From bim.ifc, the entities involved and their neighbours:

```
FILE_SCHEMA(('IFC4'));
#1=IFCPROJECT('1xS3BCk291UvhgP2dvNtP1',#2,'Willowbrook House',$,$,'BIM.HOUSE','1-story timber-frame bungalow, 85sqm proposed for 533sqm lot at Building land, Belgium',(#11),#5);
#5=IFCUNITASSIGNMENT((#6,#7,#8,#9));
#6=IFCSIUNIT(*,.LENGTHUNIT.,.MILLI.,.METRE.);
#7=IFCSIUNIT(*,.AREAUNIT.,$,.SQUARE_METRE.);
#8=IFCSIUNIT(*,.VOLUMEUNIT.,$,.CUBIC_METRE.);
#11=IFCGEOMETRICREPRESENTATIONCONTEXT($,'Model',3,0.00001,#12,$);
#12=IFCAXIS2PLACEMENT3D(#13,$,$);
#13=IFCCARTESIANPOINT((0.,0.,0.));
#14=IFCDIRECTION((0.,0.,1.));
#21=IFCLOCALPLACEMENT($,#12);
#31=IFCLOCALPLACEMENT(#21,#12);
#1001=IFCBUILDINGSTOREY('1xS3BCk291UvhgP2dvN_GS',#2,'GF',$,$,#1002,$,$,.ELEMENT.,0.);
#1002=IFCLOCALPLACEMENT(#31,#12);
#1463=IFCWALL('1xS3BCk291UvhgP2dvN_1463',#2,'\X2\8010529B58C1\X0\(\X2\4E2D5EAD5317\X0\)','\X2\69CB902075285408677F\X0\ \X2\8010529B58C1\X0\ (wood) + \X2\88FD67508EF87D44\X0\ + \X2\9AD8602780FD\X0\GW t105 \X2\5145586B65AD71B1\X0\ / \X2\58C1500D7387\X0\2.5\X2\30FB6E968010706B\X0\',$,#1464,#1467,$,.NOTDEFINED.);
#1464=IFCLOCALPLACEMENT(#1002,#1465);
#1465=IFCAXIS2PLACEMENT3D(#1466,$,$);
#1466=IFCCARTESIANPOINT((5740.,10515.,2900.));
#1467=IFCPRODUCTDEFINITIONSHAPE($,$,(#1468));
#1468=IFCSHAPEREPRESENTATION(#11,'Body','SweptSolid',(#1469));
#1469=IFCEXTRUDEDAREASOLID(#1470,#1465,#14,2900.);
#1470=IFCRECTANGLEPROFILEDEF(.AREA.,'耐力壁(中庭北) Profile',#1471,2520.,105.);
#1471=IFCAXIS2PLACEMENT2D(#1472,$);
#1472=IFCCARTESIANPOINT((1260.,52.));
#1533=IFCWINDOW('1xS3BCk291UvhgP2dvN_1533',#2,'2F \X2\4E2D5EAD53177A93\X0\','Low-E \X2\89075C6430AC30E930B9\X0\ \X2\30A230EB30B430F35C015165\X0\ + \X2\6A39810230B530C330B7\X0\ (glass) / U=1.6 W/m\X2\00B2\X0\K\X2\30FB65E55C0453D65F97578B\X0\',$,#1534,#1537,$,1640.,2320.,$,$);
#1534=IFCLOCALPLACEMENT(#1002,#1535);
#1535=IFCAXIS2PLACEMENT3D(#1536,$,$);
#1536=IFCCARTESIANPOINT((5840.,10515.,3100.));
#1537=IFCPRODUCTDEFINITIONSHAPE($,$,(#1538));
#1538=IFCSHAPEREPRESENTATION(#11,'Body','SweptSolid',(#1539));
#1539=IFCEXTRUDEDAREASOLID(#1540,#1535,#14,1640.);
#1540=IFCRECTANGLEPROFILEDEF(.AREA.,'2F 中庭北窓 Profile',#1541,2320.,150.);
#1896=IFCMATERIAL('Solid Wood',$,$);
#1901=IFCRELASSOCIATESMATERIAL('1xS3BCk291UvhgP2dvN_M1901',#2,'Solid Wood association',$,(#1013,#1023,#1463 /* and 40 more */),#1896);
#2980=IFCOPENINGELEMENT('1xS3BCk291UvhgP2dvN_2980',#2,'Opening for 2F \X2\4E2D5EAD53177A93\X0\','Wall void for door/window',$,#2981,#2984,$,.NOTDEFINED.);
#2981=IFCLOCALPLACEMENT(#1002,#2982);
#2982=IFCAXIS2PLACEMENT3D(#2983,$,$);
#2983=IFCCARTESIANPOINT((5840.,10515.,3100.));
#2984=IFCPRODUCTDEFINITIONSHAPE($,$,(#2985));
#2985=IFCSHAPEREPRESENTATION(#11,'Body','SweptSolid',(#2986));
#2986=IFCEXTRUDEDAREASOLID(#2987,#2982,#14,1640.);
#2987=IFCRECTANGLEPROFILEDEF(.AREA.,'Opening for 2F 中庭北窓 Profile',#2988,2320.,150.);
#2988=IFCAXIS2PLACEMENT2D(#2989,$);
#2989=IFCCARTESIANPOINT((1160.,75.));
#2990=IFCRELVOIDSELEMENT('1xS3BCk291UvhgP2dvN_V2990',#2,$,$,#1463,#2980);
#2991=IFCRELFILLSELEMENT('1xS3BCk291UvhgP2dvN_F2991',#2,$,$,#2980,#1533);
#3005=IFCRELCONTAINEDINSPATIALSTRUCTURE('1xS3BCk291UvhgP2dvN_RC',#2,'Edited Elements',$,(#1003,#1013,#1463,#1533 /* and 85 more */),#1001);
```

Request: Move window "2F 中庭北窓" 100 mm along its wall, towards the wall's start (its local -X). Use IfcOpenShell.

```python
import ifcopenshell
import ifcopenshell.api.geometry
import ifcopenshell.util.placement
import ifcopenshell.util.unit

model = ifcopenshell.open("bim.ifc")
unit_scale = ifcopenshell.util.unit.calculate_unit_scale(model)

window = model.by_guid("1xS3BCk291UvhgP2dvN_1533")
opening = window.FillsVoids[0].RelatingOpeningElement
wall = opening.VoidsElements[0].RelatingBuildingElement

wall_matrix = ifcopenshell.util.placement.get_local_placement(wall.ObjectPlacement)
shift = wall_matrix[:3, 0] * -0.1 / unit_scale
before = ifcopenshell.util.placement.get_local_placement(window.ObjectPlacement)[:3, 3].copy()

# The window is not placed relative to its opening, so move both.
for product in (opening, window):
    matrix = ifcopenshell.util.placement.get_local_placement(product.ObjectPlacement)
    matrix[:3, 3] += shift
    ifcopenshell.api.geometry.edit_object_placement(model, product=product, matrix=matrix, is_si=False)

after = ifcopenshell.util.placement.get_local_placement(window.ObjectPlacement)[:3, 3]
print("window moved by", (after - before).round(3) + 0.0)

model.write("bim_v2.ifc")
```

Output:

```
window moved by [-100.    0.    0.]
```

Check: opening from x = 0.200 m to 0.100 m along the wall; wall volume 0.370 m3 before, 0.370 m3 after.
